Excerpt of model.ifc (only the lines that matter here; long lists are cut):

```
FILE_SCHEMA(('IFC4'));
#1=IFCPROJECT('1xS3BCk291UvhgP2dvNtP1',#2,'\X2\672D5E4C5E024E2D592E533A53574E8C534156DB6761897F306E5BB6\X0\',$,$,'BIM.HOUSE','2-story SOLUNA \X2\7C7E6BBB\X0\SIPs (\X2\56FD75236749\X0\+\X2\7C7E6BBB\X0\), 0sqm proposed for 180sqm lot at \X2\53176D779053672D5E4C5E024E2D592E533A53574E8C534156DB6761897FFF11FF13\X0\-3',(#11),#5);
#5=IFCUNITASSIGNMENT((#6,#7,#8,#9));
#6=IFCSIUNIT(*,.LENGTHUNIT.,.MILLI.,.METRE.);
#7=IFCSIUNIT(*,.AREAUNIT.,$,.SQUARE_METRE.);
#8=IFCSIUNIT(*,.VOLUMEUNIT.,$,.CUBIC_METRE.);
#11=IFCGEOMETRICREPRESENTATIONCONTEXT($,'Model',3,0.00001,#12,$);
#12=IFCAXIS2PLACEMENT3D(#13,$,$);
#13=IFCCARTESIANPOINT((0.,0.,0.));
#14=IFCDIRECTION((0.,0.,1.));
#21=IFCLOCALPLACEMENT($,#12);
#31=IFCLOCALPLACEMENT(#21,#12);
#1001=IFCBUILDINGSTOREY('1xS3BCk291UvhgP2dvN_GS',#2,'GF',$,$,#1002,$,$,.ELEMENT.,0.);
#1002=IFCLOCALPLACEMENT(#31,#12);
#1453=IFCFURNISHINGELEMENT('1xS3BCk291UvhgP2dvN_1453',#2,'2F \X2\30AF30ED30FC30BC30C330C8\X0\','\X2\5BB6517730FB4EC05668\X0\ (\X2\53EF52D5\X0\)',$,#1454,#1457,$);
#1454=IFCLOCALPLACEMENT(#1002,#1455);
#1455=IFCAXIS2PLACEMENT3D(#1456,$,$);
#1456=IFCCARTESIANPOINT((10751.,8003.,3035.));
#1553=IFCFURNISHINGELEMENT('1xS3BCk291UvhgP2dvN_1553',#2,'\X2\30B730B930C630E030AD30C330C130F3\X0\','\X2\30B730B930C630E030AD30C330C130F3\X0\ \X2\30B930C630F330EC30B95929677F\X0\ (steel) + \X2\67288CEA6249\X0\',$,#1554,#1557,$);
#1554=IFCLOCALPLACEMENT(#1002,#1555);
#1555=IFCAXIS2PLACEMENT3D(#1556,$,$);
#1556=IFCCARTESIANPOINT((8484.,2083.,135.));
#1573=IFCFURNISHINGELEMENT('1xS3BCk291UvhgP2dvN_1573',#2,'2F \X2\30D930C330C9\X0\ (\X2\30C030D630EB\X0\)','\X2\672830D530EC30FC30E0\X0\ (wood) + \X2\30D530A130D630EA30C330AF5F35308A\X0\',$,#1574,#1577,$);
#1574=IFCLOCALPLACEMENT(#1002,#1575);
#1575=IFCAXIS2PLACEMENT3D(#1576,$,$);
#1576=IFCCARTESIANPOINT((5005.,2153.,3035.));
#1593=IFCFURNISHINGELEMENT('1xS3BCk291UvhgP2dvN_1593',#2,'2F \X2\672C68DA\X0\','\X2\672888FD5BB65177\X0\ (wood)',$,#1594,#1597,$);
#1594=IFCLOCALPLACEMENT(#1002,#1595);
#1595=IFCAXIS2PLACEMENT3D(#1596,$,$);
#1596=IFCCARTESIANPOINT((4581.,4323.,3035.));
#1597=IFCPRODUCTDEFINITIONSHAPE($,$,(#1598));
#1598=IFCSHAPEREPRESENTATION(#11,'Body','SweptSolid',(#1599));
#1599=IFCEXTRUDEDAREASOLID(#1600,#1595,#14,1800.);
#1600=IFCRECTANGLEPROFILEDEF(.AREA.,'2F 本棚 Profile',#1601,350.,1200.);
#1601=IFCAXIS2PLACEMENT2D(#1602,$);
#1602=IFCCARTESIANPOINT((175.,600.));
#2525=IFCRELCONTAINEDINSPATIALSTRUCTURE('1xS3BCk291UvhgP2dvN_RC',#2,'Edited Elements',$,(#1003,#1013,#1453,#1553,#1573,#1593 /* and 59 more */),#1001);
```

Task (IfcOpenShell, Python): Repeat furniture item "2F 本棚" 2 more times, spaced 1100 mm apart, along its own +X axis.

```python
import ifcopenshell
import ifcopenshell.api.geometry
import ifcopenshell.api.root
import ifcopenshell.util.element
import ifcopenshell.util.placement
import ifcopenshell.util.unit

model = ifcopenshell.open("model.ifc")
unit_scale = ifcopenshell.util.unit.calculate_unit_scale(model)


def reuse_history(source, copy):
    """copy_class also copies each property set's owner history, people and application; keep the originals."""
    for rel in copy.IsDefinedBy:
        if rel.is_a("IfcRelDefinesByProperties") and (history := rel.RelatingPropertyDefinition.OwnerHistory):
            rel.RelatingPropertyDefinition.OwnerHistory = source.OwnerHistory
            ifcopenshell.util.element.remove_deep2(model, history)


source = model.by_guid("1xS3BCk291UvhgP2dvN_1593")
base = ifcopenshell.util.placement.get_local_placement(source.ObjectPlacement)
step = base[:3, 0] * 1.1 / unit_scale

for i in range(1, 3):
    copy = ifcopenshell.api.root.copy_class(model, product=source)
    copy.Representation = ifcopenshell.util.element.copy_deep(
        model, source.Representation, exclude=["IfcGeometricRepresentationContext", "IfcRepresentationMap"]
    )
    reuse_history(source, copy)
    matrix = base.copy()
    matrix[:3, 3] += i * step
    print("added at", matrix[:3, 3].round(3) + 0.0)
    ifcopenshell.api.geometry.edit_object_placement(model, product=copy, matrix=matrix, is_si=False)

model.write("model_updated.ifc")
```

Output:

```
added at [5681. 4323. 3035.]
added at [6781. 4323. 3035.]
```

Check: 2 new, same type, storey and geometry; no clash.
